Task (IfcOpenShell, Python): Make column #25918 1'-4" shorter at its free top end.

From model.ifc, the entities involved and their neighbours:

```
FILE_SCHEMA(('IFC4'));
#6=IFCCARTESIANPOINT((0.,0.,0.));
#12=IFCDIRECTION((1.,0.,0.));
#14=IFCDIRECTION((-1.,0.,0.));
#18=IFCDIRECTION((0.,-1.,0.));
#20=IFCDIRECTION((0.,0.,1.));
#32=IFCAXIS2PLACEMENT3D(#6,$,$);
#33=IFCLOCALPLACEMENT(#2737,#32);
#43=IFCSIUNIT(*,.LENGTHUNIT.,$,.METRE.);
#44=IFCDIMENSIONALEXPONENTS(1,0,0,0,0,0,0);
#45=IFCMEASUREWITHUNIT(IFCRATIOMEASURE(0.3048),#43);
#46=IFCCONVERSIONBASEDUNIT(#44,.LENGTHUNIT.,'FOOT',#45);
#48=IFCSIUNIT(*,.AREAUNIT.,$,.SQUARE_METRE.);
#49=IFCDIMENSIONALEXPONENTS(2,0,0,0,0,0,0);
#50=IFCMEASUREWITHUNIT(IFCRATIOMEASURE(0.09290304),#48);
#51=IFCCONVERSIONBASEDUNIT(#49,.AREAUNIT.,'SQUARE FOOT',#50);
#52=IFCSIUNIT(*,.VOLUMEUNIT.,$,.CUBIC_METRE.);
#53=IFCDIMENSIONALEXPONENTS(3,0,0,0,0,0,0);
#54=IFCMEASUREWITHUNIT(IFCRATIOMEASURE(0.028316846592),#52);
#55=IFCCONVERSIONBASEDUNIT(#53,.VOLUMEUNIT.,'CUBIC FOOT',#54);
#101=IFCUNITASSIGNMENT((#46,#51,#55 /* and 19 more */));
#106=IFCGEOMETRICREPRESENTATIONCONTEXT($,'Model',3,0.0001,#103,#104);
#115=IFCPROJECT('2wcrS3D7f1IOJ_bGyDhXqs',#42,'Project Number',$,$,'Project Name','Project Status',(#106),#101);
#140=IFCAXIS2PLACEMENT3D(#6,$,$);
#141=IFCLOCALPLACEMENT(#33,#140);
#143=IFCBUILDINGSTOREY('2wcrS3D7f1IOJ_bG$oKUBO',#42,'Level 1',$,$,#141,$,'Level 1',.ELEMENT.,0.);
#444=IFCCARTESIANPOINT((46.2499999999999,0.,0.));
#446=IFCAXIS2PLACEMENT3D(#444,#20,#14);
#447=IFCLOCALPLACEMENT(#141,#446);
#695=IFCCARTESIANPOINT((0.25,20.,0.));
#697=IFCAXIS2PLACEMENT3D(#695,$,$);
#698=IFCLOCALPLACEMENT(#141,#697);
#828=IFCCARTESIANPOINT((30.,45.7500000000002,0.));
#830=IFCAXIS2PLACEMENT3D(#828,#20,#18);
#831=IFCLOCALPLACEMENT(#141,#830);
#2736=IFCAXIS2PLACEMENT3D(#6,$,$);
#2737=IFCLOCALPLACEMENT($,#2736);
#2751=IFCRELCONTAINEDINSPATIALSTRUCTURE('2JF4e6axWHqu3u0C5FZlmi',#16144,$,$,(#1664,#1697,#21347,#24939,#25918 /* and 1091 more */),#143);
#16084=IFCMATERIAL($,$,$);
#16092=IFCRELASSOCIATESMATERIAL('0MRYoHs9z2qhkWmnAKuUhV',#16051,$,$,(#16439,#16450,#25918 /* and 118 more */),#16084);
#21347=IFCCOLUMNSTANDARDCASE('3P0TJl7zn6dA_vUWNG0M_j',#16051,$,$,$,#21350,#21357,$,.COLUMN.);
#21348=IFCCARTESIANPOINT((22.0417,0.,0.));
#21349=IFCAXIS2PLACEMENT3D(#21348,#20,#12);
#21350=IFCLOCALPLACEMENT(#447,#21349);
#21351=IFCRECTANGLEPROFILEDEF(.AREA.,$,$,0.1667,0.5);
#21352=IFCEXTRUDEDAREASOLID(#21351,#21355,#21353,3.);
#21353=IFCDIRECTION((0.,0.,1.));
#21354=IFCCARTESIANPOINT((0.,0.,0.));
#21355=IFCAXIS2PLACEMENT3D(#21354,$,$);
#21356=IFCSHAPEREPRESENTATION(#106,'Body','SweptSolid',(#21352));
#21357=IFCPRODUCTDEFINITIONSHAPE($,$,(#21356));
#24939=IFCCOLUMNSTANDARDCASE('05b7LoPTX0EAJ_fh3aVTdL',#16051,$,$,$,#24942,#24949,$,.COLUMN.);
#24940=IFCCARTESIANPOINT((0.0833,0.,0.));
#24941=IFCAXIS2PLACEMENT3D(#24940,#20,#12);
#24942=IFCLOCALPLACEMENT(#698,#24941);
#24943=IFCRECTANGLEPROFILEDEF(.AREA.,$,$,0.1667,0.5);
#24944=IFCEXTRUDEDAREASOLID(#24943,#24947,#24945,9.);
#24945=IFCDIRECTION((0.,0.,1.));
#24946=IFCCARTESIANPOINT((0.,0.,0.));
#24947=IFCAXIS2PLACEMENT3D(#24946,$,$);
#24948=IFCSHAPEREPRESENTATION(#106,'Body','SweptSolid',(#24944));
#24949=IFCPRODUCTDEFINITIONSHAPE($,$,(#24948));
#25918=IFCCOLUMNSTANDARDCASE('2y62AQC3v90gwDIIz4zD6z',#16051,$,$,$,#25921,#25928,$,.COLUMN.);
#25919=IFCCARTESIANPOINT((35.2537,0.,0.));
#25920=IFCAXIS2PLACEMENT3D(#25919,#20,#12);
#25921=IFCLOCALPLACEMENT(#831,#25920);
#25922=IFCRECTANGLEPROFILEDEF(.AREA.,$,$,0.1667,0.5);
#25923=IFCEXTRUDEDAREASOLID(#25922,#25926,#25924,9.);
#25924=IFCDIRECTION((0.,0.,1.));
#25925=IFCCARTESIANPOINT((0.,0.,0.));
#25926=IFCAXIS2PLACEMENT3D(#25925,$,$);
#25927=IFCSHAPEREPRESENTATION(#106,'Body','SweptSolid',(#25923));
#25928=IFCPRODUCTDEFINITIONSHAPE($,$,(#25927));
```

```python
import ifcopenshell
import ifcopenshell.util.unit

model = ifcopenshell.open("model.ifc")
unit_scale = ifcopenshell.util.unit.calculate_unit_scale(model)

member = model.by_guid("2y62AQC3v90gwDIIz4zD6z")
change = -16 * 0.0254 / unit_scale

# The extrusion runs towards the end named, so only its depth changes.
body = next(r for r in member.Representation.Representations if r.RepresentationIdentifier == "Body")
solid = body.Items[0]
old_length = solid.Depth
solid.Depth += change

print(f"length {old_length:g} -> {solid.Depth:g}")

model.write("model_rev.ifc")
```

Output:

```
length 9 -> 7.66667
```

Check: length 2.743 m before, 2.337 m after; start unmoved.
